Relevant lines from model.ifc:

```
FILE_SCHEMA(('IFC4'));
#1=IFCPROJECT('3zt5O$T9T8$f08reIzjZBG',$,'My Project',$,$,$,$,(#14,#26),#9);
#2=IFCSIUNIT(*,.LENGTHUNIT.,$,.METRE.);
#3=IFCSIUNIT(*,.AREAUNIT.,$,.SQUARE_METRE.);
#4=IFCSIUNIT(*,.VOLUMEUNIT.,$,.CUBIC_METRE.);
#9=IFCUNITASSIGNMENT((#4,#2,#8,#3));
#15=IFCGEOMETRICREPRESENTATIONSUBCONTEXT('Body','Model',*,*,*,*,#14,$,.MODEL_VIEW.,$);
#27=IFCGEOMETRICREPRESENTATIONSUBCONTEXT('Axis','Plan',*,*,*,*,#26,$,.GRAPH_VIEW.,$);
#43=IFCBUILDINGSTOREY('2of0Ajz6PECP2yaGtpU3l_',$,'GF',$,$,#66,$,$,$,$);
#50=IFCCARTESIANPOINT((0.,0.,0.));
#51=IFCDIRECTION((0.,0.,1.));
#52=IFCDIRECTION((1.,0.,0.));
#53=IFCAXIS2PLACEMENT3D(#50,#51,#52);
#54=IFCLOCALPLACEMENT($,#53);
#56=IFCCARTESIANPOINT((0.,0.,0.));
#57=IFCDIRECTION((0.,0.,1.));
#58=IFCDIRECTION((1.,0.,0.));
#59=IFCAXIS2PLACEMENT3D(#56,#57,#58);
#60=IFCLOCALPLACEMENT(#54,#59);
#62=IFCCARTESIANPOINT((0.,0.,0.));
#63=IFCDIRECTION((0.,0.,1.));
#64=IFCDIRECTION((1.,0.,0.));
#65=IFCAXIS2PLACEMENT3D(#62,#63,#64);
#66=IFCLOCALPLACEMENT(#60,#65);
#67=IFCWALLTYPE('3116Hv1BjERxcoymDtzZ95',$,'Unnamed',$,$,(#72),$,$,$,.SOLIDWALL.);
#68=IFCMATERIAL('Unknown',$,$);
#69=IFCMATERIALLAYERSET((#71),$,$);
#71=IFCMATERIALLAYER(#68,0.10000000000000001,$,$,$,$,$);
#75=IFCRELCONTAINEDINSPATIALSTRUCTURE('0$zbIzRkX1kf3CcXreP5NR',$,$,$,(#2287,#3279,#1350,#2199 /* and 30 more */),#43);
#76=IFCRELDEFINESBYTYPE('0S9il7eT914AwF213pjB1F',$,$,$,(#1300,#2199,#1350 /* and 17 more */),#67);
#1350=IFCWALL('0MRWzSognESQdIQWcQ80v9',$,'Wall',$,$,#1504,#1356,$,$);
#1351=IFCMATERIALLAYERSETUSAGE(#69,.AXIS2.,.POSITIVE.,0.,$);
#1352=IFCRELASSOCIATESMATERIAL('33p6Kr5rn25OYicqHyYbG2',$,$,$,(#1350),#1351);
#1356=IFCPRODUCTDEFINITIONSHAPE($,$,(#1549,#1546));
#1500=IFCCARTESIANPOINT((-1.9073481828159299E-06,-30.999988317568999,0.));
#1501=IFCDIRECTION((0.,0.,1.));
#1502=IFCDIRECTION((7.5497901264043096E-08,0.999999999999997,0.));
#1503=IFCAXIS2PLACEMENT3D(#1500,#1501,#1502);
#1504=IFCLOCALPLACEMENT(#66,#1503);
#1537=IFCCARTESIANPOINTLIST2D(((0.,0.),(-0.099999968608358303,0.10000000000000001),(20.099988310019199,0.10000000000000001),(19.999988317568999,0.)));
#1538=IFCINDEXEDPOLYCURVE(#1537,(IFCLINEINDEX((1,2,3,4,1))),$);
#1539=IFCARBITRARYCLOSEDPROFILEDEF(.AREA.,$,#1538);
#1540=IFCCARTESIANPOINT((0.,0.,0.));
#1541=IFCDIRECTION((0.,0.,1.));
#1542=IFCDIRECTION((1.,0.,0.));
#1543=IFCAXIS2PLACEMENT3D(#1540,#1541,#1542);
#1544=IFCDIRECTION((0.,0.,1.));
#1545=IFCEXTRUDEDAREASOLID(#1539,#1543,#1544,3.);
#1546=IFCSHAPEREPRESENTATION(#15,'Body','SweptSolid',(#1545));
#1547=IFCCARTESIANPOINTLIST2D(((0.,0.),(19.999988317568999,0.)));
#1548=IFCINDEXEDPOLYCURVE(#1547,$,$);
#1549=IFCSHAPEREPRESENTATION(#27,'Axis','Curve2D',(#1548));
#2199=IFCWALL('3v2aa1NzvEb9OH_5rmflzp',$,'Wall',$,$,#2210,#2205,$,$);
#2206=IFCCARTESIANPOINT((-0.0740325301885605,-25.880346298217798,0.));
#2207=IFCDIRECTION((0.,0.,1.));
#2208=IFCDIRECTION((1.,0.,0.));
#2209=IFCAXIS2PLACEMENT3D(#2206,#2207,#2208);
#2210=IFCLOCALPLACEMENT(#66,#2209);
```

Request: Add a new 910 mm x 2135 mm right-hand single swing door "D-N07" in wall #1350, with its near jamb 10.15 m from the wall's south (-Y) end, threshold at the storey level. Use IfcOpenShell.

```python
import numpy as np
import ifcopenshell
import ifcopenshell.api.feature
import ifcopenshell.api.geometry
import ifcopenshell.api.root
import ifcopenshell.api.spatial
import ifcopenshell.geom
import ifcopenshell.util.element
import ifcopenshell.util.placement
import ifcopenshell.util.representation
import ifcopenshell.util.shape
import ifcopenshell.util.unit

model = ifcopenshell.open("model.ifc")
unit_scale = ifcopenshell.util.unit.calculate_unit_scale(model)
settings = ifcopenshell.geom.settings()


def volume(element):
    """Net volume in cubic metres, openings subtracted."""
    shape = ifcopenshell.geom.create_shape(settings, element)
    return ifcopenshell.util.shape.get_volume(shape.geometry)


wall = model.by_guid("0MRWzSognESQdIQWcQ80v9")
storey = ifcopenshell.util.element.get_container(wall, ifc_class="IfcBuildingStorey")
context = ifcopenshell.util.representation.get_context(model, "Model", "Body", "MODEL_VIEW")
before = volume(wall)

width, height, from_end, sill = 0.91, 2.135, 10.15, 0.0  # metres

# The wall runs along its own X axis, and the end named is its -X end.
wall_shape = ifcopenshell.geom.create_shape(settings, wall)
x, y, z = ifcopenshell.util.shape.get_vertices(wall_shape.geometry).T
start = x.min() + from_end
face, thickness = float(y.min()), float(y.max() - y.min())
wall_matrix = ifcopenshell.util.placement.get_local_placement(wall.ObjectPlacement)
level = ifcopenshell.util.placement.get_local_placement(storey.ObjectPlacement)[2, 3]


def in_wall(x, y):
    """Placement at x, y metres in the wall's axes, at sill height."""
    matrix = wall_matrix.copy()
    matrix[:, 3] = wall_matrix @ np.array([x / unit_scale, y / unit_scale, 0.0, 1.0])
    matrix[2, 3] = level + sill / unit_scale
    return matrix


# Opening: a box that overshoots both wall faces by 50 mm.
opening = ifcopenshell.api.root.create_entity(model, ifc_class="IfcOpeningElement", predefined_type="OPENING")
box = ifcopenshell.api.geometry.add_wall_representation(
    model, context=context, length=width, height=height, thickness=thickness + 0.1
)
ifcopenshell.api.geometry.assign_representation(model, product=opening, representation=box)
ifcopenshell.api.geometry.edit_object_placement(model, product=opening, matrix=in_wall(start, face - 0.05), is_si=False)
ifcopenshell.api.feature.add_feature(model, feature=opening, element=wall)

door = ifcopenshell.api.root.create_entity(model, ifc_class="IfcDoor", name="D-N07", predefined_type="DOOR")
door.OverallWidth, door.OverallHeight = width / unit_scale, height / unit_scale
door.OperationType = "SINGLE_SWING_RIGHT"
body = ifcopenshell.api.geometry.add_door_representation(
    model,
    context=context,
    overall_width=door.OverallWidth,
    overall_height=door.OverallHeight,
    operation_type="SINGLE_SWING_RIGHT",
    lining_properties={"LiningDepth": thickness / unit_scale, "ThresholdDepth": thickness / unit_scale},
)
ifcopenshell.api.geometry.assign_representation(model, product=door, representation=body)
ifcopenshell.api.spatial.assign_container(model, products=[door], relating_structure=storey)
ifcopenshell.api.feature.add_filling(model, opening=opening, element=door)

# The lining spans the wall, so the door starts at the wall face.
ifcopenshell.api.geometry.edit_object_placement(model, product=door, matrix=in_wall(start, face), is_si=False)

after = volume(wall)

print(f"wall volume {before:.3f} -> {after:.3f} m3")

model.write("model-out.ifc")
```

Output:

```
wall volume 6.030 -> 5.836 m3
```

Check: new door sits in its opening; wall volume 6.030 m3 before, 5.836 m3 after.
